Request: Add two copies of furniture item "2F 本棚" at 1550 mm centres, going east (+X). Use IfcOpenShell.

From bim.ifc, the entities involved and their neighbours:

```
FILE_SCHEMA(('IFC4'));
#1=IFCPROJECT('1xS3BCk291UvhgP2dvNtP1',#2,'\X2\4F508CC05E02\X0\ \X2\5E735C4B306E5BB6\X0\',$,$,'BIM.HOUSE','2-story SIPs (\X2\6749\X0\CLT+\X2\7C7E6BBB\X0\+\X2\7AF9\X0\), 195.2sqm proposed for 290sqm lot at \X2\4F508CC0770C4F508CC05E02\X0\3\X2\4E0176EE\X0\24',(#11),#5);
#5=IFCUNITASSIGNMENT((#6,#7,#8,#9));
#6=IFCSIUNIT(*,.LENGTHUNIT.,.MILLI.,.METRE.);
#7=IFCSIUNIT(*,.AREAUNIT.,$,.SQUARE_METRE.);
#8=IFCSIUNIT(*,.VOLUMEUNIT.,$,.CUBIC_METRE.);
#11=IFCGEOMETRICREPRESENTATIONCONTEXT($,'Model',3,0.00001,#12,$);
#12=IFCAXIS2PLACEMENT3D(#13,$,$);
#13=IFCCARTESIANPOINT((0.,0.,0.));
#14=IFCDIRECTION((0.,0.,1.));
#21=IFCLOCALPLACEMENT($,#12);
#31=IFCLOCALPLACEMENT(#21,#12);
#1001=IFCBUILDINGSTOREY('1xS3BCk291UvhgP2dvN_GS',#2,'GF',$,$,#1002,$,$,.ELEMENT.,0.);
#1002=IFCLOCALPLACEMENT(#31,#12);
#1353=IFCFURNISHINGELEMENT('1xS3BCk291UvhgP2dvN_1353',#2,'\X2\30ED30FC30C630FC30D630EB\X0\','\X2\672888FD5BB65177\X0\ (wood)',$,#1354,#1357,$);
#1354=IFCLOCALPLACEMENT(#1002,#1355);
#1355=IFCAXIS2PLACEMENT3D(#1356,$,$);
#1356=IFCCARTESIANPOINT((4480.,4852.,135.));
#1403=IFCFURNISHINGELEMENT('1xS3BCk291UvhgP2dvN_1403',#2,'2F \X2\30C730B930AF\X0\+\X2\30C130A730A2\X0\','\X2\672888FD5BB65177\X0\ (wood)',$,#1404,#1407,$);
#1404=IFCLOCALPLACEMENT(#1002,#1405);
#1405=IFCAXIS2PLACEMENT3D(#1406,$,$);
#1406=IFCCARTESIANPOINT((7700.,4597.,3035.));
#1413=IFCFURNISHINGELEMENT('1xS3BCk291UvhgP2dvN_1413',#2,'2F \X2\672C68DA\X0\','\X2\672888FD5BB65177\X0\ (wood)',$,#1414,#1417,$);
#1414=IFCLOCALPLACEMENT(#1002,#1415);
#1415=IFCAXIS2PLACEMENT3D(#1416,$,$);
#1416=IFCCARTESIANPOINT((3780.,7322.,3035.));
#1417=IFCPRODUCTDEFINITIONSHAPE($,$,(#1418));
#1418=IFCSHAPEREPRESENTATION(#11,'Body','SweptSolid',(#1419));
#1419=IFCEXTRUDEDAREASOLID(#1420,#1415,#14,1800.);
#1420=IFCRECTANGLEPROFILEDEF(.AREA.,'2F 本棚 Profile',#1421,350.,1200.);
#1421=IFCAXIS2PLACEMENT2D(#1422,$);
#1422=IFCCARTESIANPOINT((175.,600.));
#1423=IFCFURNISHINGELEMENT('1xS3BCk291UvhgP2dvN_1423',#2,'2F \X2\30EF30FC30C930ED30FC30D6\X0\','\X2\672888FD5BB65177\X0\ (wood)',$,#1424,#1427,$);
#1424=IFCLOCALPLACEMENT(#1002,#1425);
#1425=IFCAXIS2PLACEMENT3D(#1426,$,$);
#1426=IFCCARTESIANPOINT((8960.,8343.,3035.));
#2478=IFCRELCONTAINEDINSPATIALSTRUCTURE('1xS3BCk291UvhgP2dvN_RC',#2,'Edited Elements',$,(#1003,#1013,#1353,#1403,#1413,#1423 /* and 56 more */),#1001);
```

```python
import numpy as np
import ifcopenshell
import ifcopenshell.api.geometry
import ifcopenshell.api.root
import ifcopenshell.util.element
import ifcopenshell.util.placement
import ifcopenshell.util.unit

model = ifcopenshell.open("bim.ifc")
unit_scale = ifcopenshell.util.unit.calculate_unit_scale(model)


def reuse_history(source, copy):
    """copy_class also copies each property set's owner history, people and application; keep the originals."""
    for rel in copy.IsDefinedBy:
        if rel.is_a("IfcRelDefinesByProperties") and (history := rel.RelatingPropertyDefinition.OwnerHistory):
            rel.RelatingPropertyDefinition.OwnerHistory = source.OwnerHistory
            ifcopenshell.util.element.remove_deep2(model, history)


source = model.by_guid("1xS3BCk291UvhgP2dvN_1413")
base = ifcopenshell.util.placement.get_local_placement(source.ObjectPlacement)
step = np.array([1.0, 0.0, 0.0]) * 1.55 / unit_scale

for i in range(1, 3):
    copy = ifcopenshell.api.root.copy_class(model, product=source)
    copy.Representation = ifcopenshell.util.element.copy_deep(
        model, source.Representation, exclude=["IfcGeometricRepresentationContext", "IfcRepresentationMap"]
    )
    reuse_history(source, copy)
    matrix = base.copy()
    matrix[:3, 3] += i * step
    print("added at", matrix[:3, 3].round(3) + 0.0)
    ifcopenshell.api.geometry.edit_object_placement(model, product=copy, matrix=matrix, is_si=False)

model.write("bim_updated.ifc")
```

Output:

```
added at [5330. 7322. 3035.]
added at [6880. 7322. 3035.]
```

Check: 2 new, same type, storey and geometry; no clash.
